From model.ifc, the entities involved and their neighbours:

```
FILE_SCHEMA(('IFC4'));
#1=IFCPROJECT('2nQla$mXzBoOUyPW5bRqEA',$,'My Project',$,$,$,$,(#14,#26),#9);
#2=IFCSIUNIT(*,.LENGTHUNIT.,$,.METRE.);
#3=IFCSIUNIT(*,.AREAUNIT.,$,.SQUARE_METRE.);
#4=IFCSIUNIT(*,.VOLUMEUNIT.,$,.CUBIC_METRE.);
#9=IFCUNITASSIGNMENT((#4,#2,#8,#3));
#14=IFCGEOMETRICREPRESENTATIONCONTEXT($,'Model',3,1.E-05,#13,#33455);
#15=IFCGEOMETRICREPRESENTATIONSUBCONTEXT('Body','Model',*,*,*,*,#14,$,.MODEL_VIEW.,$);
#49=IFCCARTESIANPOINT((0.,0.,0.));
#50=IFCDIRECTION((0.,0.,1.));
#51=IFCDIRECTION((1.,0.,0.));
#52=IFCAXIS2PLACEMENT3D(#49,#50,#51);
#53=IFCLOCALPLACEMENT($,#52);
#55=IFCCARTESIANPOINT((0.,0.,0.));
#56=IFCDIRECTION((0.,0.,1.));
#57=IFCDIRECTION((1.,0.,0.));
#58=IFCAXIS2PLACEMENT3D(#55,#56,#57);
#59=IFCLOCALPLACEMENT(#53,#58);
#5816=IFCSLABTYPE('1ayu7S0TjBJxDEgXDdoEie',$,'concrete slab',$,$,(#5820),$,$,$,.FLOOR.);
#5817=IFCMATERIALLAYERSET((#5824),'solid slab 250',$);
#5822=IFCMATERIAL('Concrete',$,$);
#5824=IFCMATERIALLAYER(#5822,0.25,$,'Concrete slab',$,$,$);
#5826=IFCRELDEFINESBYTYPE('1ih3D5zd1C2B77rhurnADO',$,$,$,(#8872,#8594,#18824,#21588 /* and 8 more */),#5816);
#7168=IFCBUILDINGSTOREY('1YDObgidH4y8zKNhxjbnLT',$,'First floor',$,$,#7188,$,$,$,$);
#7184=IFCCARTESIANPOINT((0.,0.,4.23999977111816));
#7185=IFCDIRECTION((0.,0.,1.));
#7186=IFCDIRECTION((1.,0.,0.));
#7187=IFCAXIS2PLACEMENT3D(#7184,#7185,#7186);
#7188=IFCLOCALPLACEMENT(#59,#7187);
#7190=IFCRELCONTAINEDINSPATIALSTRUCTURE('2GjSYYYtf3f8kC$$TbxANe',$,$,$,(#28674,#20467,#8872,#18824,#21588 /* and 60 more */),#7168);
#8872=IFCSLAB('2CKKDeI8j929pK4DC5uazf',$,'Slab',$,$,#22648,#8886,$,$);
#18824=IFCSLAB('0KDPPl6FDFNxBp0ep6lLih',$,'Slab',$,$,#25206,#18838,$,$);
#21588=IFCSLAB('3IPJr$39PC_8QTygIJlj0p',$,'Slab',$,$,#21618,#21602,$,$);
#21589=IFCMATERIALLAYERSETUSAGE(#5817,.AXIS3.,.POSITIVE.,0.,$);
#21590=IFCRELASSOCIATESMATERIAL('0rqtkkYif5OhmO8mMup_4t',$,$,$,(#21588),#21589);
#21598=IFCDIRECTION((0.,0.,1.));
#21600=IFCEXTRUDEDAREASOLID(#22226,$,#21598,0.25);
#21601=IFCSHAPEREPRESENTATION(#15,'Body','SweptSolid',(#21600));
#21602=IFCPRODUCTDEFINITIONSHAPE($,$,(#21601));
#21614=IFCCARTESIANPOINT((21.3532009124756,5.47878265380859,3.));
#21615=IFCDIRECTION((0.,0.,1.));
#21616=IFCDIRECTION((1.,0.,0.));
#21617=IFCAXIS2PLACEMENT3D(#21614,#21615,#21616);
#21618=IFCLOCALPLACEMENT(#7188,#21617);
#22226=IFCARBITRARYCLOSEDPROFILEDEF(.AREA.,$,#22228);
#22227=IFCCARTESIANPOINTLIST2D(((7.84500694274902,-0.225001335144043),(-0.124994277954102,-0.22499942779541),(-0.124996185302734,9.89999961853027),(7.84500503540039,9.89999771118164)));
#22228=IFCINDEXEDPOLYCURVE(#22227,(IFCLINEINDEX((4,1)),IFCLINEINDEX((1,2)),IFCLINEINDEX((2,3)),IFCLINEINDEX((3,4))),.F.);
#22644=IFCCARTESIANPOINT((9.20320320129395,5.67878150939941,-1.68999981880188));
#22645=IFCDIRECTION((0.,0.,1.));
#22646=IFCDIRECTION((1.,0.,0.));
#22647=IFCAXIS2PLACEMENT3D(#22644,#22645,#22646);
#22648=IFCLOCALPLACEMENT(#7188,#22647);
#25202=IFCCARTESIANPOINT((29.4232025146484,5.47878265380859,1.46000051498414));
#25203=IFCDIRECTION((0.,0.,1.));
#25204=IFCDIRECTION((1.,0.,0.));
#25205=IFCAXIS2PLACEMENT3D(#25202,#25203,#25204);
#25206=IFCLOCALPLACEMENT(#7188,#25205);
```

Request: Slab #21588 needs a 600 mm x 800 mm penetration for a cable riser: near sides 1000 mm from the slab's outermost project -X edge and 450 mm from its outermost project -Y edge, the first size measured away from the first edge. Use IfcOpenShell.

```python
import numpy as np
import ifcopenshell
import ifcopenshell.api.feature
import ifcopenshell.api.geometry
import ifcopenshell.api.root
import ifcopenshell.geom
import ifcopenshell.util.placement
import ifcopenshell.util.representation
import ifcopenshell.util.shape
import ifcopenshell.util.unit

model = ifcopenshell.open("model.ifc")
unit_scale = ifcopenshell.util.unit.calculate_unit_scale(model)
settings = ifcopenshell.geom.settings()


def volume(element):
    """Net volume in cubic metres, openings subtracted."""
    shape = ifcopenshell.geom.create_shape(settings, element)
    return ifcopenshell.util.shape.get_volume(shape.geometry)


slab = model.by_guid("3IPJr$39PC_8QTygIJlj0p")
before = volume(slab)

# Extent in the slab's own axes, in metres. The edges named are its -X and -Y sides.
slab_shape = ifcopenshell.geom.create_shape(settings, slab)
vertices = ifcopenshell.util.shape.get_vertices(slab_shape.geometry)
x_min, y_min, bottom = vertices.min(axis=0)
top = vertices[:, 2].max()

opening = ifcopenshell.api.root.create_entity(model, ifc_class="IfcOpeningElement", name="Cable riser opening", predefined_type="OPENING")
context = ifcopenshell.util.representation.get_context(model, "Model", "Body", "MODEL_VIEW")
width, depth = 0.6, 0.8
outline = [(0.0, 0.0), (width, 0.0), (width, depth), (0.0, depth), (0.0, 0.0)]
# Overshoot both faces by 50 mm so the cut is clean.
shape = ifcopenshell.api.geometry.add_slab_representation(
    model, context=context, depth=top - bottom + 0.1, polyline=outline
)
ifcopenshell.api.geometry.assign_representation(model, product=opening, representation=shape)

matrix = ifcopenshell.util.placement.get_local_placement(slab.ObjectPlacement)
matrix[:, 3] = matrix @ np.append(np.array([x_min + 1, y_min + 0.45, bottom - 0.05]) / unit_scale, 1.0)
ifcopenshell.api.geometry.edit_object_placement(model, product=opening, matrix=matrix, is_si=False)
ifcopenshell.api.feature.add_feature(model, feature=opening, element=slab)

after = volume(slab)

print(f"slab volume {before:.3f} -> {after:.3f} m3")

model.write("model_updated.ifc")
```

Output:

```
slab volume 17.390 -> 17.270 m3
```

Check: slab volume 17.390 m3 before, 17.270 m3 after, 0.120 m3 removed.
